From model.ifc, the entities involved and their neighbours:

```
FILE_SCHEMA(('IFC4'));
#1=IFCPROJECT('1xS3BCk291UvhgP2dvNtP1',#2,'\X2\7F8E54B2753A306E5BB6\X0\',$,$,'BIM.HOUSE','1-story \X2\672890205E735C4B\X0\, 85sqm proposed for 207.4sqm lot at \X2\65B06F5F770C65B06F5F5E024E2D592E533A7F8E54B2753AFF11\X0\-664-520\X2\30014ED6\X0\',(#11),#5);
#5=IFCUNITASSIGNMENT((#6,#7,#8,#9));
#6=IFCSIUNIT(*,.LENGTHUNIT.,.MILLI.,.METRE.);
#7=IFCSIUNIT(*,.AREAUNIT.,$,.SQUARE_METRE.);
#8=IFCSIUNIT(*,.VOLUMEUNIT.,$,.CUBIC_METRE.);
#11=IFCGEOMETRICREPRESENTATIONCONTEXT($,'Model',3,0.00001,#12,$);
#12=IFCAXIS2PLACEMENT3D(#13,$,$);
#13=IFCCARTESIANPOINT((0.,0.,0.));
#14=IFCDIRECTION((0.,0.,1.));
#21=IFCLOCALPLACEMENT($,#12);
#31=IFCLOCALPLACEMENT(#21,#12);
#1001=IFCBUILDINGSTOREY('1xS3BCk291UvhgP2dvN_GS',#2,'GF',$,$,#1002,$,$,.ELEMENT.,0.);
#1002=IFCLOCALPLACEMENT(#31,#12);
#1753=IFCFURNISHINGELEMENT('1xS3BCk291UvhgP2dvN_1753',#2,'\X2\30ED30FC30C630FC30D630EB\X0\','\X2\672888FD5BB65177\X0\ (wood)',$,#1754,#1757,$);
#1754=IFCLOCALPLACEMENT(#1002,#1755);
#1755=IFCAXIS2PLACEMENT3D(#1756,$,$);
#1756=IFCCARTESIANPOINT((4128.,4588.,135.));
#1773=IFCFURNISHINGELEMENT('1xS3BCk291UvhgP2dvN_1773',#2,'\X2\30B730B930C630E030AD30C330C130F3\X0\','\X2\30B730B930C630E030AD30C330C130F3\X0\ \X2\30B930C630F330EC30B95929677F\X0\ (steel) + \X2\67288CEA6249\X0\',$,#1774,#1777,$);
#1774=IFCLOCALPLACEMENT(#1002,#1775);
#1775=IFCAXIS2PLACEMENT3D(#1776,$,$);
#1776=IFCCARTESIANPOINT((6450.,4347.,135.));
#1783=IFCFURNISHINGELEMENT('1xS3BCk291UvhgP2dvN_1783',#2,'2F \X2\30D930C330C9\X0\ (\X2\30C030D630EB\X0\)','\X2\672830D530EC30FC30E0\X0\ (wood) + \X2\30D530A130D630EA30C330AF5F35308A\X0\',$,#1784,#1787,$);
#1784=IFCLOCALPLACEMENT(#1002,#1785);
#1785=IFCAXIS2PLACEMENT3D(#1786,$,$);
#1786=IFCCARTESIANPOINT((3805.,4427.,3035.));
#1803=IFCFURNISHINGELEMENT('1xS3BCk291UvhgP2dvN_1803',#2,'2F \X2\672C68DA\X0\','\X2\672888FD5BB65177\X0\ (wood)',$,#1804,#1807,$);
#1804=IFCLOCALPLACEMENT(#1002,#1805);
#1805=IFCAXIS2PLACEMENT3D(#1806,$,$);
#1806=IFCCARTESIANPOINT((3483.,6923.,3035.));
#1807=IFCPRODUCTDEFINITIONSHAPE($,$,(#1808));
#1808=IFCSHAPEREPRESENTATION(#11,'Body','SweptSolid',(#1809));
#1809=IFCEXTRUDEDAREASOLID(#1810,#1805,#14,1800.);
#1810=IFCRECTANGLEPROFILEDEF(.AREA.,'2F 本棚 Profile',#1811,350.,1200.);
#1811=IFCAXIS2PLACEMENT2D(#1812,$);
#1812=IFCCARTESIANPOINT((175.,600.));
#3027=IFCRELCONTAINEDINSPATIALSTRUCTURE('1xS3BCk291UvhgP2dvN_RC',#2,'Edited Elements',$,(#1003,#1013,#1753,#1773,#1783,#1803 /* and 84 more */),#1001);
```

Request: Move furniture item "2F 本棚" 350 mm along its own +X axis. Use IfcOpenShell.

```python
import ifcopenshell
import ifcopenshell.api.geometry
import ifcopenshell.util.placement
import ifcopenshell.util.unit

model = ifcopenshell.open("model.ifc")
unit_scale = ifcopenshell.util.unit.calculate_unit_scale(model)

item = model.by_guid("1xS3BCk291UvhgP2dvN_1803")
matrix = ifcopenshell.util.placement.get_local_placement(item.ObjectPlacement)
matrix[:3, 3] += matrix[:3, 0] * 0.35 / unit_scale
ifcopenshell.api.geometry.edit_object_placement(model, product=item, matrix=matrix, is_si=False)

print(ifcopenshell.util.placement.get_local_placement(item.ObjectPlacement).round(3) + 0.0)

model.write("model_v2.ifc")
```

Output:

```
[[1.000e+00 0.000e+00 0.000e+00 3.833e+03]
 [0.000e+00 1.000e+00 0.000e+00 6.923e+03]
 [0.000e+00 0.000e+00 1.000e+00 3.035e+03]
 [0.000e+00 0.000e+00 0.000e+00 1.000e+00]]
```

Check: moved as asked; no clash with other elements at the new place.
